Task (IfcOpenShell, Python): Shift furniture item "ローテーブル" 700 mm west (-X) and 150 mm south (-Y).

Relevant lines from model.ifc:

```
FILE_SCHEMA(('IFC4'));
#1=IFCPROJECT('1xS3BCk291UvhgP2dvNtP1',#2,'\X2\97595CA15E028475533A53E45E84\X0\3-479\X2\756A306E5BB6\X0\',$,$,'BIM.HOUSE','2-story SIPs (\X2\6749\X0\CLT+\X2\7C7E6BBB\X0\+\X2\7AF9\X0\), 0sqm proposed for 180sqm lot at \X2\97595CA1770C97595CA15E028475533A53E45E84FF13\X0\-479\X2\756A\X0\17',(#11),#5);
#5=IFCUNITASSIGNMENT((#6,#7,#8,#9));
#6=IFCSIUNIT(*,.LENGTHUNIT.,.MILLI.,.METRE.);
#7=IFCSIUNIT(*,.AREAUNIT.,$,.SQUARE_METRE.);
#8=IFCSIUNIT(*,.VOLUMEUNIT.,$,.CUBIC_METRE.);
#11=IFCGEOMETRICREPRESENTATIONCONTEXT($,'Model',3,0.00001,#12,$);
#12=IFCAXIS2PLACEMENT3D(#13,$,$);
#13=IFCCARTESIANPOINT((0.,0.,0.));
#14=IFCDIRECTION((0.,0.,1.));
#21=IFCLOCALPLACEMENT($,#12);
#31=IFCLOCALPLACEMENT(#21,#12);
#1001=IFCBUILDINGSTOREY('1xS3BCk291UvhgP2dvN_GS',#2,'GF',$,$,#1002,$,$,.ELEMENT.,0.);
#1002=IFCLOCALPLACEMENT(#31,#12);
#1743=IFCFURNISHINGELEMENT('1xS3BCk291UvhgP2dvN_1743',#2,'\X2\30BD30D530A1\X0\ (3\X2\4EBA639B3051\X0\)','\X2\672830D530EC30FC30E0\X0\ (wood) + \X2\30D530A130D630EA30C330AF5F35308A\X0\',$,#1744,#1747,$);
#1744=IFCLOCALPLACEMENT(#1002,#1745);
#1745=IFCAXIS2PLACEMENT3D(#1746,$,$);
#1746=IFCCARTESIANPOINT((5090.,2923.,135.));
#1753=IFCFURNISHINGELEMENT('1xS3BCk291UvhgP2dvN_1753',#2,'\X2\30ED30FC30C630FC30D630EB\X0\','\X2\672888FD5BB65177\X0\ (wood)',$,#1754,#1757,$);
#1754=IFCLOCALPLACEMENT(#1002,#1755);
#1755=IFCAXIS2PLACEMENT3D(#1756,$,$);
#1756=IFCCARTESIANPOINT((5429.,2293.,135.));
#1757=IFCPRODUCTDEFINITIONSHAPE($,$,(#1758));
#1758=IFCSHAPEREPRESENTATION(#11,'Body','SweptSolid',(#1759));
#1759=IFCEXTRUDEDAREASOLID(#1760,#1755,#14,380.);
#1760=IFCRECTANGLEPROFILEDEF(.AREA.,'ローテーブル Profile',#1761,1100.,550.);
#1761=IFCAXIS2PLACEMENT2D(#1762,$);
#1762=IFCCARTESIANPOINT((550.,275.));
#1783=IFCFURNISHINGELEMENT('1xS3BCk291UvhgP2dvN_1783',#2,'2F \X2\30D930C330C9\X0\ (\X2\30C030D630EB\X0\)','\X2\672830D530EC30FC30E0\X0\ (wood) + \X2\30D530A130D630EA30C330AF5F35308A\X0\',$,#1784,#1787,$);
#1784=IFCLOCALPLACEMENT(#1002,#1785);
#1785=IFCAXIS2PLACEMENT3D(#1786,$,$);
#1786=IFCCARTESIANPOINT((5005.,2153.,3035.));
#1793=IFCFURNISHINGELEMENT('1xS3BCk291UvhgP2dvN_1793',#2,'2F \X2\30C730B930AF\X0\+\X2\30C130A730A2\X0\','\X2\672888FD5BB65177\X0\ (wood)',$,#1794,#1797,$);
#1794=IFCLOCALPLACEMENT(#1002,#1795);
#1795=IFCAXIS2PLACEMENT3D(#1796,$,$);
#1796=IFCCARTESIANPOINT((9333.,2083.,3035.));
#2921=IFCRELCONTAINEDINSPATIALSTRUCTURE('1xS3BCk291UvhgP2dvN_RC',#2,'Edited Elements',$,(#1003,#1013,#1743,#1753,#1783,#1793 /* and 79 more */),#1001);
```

```python
import ifcopenshell
import ifcopenshell.api.geometry
import ifcopenshell.util.placement
import ifcopenshell.util.unit

model = ifcopenshell.open("model.ifc")
unit_scale = ifcopenshell.util.unit.calculate_unit_scale(model)

item = model.by_id(1753)
matrix = ifcopenshell.util.placement.get_local_placement(item.ObjectPlacement)
matrix[0, 3] -= 0.7 / unit_scale
matrix[1, 3] -= 0.15 / unit_scale
ifcopenshell.api.geometry.edit_object_placement(model, product=item, matrix=matrix, is_si=False)

print(ifcopenshell.util.placement.get_local_placement(item.ObjectPlacement).round(3) + 0.0)

model.write("model_v2.ifc")
```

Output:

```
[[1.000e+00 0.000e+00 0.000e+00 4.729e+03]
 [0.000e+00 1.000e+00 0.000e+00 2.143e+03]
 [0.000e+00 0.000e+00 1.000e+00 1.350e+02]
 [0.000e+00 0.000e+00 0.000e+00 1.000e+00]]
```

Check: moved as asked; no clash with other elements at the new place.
